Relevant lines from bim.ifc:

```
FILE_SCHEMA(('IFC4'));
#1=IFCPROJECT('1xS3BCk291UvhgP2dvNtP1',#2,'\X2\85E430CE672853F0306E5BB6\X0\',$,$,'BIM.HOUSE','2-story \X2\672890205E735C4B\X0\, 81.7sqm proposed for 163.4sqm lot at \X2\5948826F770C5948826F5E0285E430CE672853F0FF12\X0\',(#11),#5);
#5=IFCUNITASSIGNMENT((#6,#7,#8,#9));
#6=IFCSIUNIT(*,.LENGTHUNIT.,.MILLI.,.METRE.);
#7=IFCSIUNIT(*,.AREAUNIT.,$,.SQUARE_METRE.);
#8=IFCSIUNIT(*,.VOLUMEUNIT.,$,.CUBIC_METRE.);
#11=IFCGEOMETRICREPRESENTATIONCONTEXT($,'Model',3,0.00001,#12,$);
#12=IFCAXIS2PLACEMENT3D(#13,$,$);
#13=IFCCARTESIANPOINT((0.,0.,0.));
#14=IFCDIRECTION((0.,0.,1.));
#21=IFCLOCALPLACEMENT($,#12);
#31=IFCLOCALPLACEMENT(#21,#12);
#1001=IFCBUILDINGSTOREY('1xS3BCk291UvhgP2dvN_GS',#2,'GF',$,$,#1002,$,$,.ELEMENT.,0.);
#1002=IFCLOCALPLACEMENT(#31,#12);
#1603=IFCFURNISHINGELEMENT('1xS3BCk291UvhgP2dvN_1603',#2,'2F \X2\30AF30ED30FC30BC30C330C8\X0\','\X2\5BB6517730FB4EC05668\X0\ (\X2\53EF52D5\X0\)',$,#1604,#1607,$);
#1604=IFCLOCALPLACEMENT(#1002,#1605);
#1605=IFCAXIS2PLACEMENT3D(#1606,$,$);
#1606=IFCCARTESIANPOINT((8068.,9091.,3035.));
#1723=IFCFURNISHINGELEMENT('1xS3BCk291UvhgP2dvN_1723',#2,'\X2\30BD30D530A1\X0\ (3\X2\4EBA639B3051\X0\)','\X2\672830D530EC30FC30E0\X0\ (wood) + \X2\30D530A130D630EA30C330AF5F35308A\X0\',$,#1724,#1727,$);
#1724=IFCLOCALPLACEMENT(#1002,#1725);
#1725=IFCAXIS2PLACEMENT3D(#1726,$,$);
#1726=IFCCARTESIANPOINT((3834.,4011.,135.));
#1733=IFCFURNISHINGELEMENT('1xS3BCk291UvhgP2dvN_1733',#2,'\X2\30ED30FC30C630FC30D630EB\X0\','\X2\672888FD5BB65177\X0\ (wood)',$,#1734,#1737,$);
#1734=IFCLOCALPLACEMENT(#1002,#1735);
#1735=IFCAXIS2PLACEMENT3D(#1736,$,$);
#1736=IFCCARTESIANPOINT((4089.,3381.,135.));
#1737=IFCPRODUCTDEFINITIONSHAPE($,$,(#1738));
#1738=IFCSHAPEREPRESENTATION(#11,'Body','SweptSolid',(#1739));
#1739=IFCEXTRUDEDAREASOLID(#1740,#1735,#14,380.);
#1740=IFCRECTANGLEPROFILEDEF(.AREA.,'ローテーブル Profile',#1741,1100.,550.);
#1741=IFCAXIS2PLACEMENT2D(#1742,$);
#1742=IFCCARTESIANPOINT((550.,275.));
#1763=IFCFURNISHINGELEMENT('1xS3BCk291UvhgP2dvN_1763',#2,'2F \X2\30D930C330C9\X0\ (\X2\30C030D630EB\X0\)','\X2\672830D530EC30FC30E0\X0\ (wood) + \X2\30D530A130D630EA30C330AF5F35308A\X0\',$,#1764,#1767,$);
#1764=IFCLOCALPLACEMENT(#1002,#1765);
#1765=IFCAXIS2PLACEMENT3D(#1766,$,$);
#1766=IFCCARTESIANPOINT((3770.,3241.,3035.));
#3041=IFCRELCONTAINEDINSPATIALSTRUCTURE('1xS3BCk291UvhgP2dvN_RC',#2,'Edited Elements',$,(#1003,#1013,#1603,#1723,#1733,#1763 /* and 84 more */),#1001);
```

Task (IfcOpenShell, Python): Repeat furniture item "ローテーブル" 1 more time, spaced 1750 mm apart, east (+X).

```python
import numpy as np
import ifcopenshell
import ifcopenshell.api.geometry
import ifcopenshell.api.root
import ifcopenshell.util.element
import ifcopenshell.util.placement
import ifcopenshell.util.unit

model = ifcopenshell.open("bim.ifc")
unit_scale = ifcopenshell.util.unit.calculate_unit_scale(model)


def reuse_history(source, copy):
    """copy_class also copies each property set's owner history, people and application; keep the originals."""
    for rel in copy.IsDefinedBy:
        if rel.is_a("IfcRelDefinesByProperties") and (history := rel.RelatingPropertyDefinition.OwnerHistory):
            rel.RelatingPropertyDefinition.OwnerHistory = source.OwnerHistory
            ifcopenshell.util.element.remove_deep2(model, history)


source = model.by_guid("1xS3BCk291UvhgP2dvN_1733")
base = ifcopenshell.util.placement.get_local_placement(source.ObjectPlacement)
step = np.array([1.0, 0.0, 0.0]) * 1.75 / unit_scale

for i in range(1, 2):
    copy = ifcopenshell.api.root.copy_class(model, product=source)
    copy.Representation = ifcopenshell.util.element.copy_deep(
        model, source.Representation, exclude=["IfcGeometricRepresentationContext", "IfcRepresentationMap"]
    )
    reuse_history(source, copy)
    matrix = base.copy()
    matrix[:3, 3] += i * step
    print("added at", matrix[:3, 3].round(3) + 0.0)
    ifcopenshell.api.geometry.edit_object_placement(model, product=copy, matrix=matrix, is_si=False)

model.write("bim_updated.ifc")
```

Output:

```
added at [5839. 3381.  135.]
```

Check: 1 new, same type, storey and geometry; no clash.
